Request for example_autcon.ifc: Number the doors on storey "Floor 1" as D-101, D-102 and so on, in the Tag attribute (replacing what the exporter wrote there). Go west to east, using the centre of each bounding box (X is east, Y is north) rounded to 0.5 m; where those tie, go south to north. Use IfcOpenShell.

First a look at what the model holds.

```python
import ifcopenshell
import ifcopenshell.util.element
import ifcopenshell.util.placement

model = ifcopenshell.open("example_autcon.ifc")
print(model.schema)
storey = next(s for s in model.by_type("IfcBuildingStorey") if s.Name == "Floor 1")
doors = [e for e in ifcopenshell.util.element.get_decomposition(storey) if e.is_a("IfcDoor")]
for e in sorted(doors, key=lambda e: e.id()):
    origin = ifcopenshell.util.placement.get_local_placement(e.ObjectPlacement)[:3, 3]
    print(e.id(), e.Tag, e.Name, origin.round(2) + 0.0, sep=" | ")
```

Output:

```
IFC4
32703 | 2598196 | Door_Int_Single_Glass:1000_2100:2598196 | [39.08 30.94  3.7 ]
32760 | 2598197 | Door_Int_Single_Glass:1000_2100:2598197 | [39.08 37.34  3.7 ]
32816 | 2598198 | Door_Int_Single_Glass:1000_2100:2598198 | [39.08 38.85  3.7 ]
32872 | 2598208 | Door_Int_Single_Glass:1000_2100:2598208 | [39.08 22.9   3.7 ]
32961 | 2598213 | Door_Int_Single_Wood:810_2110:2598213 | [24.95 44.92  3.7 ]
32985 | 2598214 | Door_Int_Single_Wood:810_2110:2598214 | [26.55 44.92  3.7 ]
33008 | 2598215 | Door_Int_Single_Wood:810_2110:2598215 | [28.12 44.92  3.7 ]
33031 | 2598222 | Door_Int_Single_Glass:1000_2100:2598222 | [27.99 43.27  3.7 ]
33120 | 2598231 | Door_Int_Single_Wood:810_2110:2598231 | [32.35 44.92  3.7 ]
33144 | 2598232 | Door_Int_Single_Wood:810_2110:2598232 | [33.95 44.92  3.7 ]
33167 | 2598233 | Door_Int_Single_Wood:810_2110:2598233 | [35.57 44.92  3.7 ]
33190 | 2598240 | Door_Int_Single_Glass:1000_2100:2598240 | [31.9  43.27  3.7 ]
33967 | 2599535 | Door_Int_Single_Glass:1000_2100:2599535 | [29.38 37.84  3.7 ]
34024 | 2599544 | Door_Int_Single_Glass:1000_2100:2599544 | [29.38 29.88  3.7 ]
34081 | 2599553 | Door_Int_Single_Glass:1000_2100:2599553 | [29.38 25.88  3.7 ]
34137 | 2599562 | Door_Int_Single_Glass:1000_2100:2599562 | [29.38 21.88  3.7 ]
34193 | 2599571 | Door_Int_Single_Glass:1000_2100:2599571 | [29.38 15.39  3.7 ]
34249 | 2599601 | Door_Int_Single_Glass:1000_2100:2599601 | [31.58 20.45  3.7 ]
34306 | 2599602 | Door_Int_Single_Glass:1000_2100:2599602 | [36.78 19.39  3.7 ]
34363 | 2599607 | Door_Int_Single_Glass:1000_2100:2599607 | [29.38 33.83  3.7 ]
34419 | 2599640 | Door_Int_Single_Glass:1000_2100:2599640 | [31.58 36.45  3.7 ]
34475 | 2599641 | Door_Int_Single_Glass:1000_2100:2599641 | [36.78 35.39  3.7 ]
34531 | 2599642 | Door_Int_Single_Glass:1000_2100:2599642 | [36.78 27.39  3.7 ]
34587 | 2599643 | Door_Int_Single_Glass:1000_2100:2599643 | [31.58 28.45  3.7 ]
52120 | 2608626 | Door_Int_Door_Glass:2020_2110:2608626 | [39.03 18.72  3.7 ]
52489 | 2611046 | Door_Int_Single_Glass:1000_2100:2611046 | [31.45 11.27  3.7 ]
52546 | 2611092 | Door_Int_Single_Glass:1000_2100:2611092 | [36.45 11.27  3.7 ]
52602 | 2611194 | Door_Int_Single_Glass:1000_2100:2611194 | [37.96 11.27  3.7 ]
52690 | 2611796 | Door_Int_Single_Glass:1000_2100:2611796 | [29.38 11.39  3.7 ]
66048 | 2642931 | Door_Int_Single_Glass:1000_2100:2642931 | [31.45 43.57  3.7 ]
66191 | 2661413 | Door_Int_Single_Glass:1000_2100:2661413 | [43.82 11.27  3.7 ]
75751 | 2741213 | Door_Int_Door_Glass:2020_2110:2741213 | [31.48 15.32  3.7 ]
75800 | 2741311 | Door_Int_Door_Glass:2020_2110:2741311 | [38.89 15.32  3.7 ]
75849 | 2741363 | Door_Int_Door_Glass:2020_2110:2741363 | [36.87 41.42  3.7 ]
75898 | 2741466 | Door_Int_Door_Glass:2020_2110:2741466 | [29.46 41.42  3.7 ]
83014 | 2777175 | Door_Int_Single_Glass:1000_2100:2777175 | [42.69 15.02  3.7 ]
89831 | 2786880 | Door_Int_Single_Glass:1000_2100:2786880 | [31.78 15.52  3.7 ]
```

```python
import ifcopenshell
import ifcopenshell.geom
import ifcopenshell.util.element
import ifcopenshell.util.shape

model = ifcopenshell.open("example_autcon.ifc")
settings = ifcopenshell.geom.settings()
settings.set("use-world-coords", True)


def centre(element):
    shape = ifcopenshell.geom.create_shape(settings, element)
    return ifcopenshell.util.shape.get_bbox_centroid(shape.geometry)


storey = next(s for s in model.by_type("IfcBuildingStorey") if s.Name == "Floor 1")
doors = [e for e in ifcopenshell.util.element.get_decomposition(storey) if e.is_a("IfcDoor")]

# Insertion points can sit at a corner or the storey origin, so sort by the geometry (in metres).
centres = {e: centre(e) for e in doors}
doors.sort(key=lambda e: (round(centres[e][0] / 0.5), centres[e][1]))

for i, e in enumerate(doors, start=1):
    number = f"D-1{i:02d}"
    e.Tag = number
    print(e.id(), number)

model.write("example_autcon_updated.ifc")
```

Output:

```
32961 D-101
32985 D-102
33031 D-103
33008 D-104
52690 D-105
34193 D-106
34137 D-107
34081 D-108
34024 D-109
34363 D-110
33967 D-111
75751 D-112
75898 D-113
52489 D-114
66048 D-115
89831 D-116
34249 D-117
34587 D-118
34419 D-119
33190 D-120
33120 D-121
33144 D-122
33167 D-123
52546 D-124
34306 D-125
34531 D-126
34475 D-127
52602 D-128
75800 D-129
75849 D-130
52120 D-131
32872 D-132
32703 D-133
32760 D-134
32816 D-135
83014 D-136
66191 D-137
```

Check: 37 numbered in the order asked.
